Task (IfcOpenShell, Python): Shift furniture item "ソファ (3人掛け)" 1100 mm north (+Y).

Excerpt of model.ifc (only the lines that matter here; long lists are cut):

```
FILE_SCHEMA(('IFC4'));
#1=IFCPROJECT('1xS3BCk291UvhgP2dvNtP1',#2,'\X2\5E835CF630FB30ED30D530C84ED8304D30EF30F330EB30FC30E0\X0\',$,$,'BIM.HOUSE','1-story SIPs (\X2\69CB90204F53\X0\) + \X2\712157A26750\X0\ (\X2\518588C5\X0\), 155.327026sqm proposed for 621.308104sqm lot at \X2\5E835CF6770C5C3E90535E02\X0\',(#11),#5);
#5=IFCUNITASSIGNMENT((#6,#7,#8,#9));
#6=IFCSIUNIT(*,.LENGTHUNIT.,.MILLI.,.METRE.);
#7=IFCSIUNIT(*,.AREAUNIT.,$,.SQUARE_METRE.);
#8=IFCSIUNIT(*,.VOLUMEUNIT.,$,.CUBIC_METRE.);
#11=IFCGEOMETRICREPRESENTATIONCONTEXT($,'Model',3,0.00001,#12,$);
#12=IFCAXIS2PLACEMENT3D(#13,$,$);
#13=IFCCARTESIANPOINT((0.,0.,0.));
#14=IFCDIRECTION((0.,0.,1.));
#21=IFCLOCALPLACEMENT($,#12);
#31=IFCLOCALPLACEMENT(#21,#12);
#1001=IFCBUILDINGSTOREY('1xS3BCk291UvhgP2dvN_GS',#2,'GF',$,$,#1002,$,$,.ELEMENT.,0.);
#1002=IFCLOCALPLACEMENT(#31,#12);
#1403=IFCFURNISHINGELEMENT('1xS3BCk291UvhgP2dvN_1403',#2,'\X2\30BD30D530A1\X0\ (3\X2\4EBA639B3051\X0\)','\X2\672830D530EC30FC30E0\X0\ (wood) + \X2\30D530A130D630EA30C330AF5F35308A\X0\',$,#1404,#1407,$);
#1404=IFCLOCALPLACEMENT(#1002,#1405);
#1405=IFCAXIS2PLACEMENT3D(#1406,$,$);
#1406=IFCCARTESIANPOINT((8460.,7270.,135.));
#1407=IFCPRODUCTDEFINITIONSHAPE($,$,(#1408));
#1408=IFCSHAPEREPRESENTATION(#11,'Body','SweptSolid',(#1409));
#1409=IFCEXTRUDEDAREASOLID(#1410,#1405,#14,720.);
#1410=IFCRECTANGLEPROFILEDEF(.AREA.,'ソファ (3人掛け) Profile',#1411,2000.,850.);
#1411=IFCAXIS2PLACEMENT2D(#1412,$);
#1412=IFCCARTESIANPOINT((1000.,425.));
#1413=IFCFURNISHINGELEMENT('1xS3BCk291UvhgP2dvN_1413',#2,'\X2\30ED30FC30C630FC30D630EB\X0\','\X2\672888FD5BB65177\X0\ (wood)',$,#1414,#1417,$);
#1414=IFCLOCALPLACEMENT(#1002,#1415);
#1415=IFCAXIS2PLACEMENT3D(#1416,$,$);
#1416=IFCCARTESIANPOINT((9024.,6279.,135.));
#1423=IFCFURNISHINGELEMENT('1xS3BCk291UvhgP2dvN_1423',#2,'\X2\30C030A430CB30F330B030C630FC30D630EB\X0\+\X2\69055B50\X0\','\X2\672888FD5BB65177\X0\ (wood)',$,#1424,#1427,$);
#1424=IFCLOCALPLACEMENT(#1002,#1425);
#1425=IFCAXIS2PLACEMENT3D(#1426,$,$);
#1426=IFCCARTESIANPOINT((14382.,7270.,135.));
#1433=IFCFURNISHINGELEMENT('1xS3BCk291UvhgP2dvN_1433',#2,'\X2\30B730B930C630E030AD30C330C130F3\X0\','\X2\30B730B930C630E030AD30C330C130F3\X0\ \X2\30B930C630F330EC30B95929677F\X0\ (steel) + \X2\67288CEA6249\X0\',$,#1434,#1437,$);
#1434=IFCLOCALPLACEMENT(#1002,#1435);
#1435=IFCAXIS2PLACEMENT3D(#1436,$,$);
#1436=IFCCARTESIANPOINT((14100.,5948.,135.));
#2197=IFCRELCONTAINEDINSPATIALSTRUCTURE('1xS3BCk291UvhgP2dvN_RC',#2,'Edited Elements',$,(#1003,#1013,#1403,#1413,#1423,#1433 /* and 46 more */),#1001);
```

```python
import ifcopenshell
import ifcopenshell.api.geometry
import ifcopenshell.util.placement
import ifcopenshell.util.unit

model = ifcopenshell.open("model.ifc")
unit_scale = ifcopenshell.util.unit.calculate_unit_scale(model)

item = model.by_id(1403)
matrix = ifcopenshell.util.placement.get_local_placement(item.ObjectPlacement)
matrix[1, 3] += 1.1 / unit_scale
ifcopenshell.api.geometry.edit_object_placement(model, product=item, matrix=matrix, is_si=False)

print(ifcopenshell.util.placement.get_local_placement(item.ObjectPlacement).round(3) + 0.0)

model.write("model_edited.ifc")
```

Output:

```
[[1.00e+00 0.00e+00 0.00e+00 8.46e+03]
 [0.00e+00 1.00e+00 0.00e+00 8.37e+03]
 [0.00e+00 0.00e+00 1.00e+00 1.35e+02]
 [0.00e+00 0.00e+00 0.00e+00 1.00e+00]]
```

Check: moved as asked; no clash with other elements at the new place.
